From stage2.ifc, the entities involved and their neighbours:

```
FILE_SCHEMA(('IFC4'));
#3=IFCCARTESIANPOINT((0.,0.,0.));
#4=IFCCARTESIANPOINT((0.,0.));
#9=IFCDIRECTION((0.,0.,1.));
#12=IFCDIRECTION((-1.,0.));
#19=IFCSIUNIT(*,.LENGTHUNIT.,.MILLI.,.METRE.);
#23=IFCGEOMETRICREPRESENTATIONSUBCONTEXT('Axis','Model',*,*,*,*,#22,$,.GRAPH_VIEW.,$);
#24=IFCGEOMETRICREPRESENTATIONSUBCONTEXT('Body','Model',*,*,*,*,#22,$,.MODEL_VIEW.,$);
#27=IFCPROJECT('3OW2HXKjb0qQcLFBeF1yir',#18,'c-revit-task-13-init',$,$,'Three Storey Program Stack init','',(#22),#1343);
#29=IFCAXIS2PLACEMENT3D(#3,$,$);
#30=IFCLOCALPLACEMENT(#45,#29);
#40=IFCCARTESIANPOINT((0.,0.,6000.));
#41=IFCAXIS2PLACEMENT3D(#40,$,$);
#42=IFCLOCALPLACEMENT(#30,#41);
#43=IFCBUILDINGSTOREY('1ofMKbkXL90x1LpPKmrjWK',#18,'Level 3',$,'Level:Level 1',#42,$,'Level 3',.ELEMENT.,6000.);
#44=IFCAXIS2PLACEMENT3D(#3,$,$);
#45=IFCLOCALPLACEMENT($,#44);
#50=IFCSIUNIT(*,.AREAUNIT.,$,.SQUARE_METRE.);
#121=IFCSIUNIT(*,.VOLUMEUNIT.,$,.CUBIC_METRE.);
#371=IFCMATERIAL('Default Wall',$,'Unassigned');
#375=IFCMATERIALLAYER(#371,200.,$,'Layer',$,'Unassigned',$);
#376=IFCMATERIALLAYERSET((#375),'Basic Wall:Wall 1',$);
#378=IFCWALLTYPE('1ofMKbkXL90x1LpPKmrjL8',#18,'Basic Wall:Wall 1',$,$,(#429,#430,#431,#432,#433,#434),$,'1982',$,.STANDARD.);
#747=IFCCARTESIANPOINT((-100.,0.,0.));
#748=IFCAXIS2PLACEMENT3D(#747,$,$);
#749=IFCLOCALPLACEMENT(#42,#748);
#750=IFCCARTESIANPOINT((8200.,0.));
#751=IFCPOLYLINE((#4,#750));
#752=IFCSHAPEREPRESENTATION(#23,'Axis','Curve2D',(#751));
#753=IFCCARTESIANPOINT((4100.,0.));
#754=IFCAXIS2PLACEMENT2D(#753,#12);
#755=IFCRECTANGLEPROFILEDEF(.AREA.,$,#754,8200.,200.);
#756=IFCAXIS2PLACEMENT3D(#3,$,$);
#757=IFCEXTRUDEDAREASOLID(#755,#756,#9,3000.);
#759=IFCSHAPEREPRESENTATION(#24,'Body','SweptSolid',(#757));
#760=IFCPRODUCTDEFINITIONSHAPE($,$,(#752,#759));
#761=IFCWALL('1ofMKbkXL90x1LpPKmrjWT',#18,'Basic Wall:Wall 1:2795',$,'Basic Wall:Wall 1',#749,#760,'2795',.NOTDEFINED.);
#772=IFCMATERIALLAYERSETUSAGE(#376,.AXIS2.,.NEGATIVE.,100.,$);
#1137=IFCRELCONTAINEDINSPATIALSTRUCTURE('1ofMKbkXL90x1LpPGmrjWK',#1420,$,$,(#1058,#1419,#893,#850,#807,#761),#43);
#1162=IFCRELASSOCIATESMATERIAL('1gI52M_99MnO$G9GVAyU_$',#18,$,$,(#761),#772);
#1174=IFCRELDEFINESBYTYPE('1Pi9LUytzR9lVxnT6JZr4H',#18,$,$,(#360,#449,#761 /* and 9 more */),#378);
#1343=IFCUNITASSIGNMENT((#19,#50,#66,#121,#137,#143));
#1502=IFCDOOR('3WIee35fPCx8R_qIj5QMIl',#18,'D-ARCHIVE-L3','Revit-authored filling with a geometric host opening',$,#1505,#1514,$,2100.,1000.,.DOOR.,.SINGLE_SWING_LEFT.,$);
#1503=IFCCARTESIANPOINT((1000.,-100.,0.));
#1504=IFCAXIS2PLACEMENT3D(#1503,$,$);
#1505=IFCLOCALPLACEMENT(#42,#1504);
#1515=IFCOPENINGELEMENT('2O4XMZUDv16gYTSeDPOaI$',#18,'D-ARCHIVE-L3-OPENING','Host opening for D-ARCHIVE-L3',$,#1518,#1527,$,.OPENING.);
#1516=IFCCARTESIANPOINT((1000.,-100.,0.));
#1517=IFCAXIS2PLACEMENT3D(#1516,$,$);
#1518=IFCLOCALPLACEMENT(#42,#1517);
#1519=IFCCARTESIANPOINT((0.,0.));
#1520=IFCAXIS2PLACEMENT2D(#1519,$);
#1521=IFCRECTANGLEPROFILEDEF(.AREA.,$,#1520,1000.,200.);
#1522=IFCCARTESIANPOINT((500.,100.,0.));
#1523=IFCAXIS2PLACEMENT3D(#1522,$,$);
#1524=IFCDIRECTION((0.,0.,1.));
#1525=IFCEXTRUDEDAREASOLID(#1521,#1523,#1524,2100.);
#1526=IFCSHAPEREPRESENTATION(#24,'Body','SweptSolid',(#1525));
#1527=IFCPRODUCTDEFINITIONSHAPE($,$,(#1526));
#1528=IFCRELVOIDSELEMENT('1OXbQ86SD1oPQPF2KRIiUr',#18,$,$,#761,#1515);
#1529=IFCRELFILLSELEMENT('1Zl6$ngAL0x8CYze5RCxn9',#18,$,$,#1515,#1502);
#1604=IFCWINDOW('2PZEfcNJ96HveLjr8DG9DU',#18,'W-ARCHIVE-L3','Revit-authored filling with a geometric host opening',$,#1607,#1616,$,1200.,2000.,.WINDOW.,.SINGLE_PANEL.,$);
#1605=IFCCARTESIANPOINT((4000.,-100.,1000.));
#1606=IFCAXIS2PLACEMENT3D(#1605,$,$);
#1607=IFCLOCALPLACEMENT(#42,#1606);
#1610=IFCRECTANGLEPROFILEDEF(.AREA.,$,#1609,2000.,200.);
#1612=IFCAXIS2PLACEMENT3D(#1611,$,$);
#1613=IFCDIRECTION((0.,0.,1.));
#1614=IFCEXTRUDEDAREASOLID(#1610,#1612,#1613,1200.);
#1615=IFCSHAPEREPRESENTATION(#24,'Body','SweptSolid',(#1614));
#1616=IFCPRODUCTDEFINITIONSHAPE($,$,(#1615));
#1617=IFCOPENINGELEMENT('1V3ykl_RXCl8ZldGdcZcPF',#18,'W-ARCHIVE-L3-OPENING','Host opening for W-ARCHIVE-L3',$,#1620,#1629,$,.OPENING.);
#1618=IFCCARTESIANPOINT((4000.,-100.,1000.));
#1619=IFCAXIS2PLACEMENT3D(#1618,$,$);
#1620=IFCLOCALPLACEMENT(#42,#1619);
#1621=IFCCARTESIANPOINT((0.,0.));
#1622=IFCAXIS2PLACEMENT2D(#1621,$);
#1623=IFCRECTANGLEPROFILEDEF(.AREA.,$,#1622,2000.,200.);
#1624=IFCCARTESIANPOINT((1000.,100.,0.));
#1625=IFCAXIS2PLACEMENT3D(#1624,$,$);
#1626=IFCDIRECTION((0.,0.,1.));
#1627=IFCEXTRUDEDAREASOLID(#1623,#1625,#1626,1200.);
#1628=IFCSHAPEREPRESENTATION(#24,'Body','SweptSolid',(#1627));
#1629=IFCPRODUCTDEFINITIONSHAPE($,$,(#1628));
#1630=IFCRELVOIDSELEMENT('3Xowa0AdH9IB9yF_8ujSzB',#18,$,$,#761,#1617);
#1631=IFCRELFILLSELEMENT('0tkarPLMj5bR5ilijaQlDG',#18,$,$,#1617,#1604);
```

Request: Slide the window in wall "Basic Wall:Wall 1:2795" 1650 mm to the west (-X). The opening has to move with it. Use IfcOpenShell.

```python
import ifcopenshell
import ifcopenshell.api.geometry
import ifcopenshell.util.placement
import ifcopenshell.util.unit

model = ifcopenshell.open("stage2.ifc")
unit_scale = ifcopenshell.util.unit.calculate_unit_scale(model)

window = model.by_guid("2PZEfcNJ96HveLjr8DG9DU")
opening = window.FillsVoids[0].RelatingOpeningElement
wall = opening.VoidsElements[0].RelatingBuildingElement

wall_matrix = ifcopenshell.util.placement.get_local_placement(wall.ObjectPlacement)
shift = wall_matrix[:3, 0] * -1.65 / unit_scale
before = ifcopenshell.util.placement.get_local_placement(window.ObjectPlacement)[:3, 3].copy()

# The window is not placed relative to its opening, so move both.
for product in (opening, window):
    matrix = ifcopenshell.util.placement.get_local_placement(product.ObjectPlacement)
    matrix[:3, 3] += shift
    ifcopenshell.api.geometry.edit_object_placement(model, product=product, matrix=matrix, is_si=False)

after = ifcopenshell.util.placement.get_local_placement(window.ObjectPlacement)[:3, 3]
print("window moved by", (after - before).round(3) + 0.0)

model.write("stage2_v2.ifc")
```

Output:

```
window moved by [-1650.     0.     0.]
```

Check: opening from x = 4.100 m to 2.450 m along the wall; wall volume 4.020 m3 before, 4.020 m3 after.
